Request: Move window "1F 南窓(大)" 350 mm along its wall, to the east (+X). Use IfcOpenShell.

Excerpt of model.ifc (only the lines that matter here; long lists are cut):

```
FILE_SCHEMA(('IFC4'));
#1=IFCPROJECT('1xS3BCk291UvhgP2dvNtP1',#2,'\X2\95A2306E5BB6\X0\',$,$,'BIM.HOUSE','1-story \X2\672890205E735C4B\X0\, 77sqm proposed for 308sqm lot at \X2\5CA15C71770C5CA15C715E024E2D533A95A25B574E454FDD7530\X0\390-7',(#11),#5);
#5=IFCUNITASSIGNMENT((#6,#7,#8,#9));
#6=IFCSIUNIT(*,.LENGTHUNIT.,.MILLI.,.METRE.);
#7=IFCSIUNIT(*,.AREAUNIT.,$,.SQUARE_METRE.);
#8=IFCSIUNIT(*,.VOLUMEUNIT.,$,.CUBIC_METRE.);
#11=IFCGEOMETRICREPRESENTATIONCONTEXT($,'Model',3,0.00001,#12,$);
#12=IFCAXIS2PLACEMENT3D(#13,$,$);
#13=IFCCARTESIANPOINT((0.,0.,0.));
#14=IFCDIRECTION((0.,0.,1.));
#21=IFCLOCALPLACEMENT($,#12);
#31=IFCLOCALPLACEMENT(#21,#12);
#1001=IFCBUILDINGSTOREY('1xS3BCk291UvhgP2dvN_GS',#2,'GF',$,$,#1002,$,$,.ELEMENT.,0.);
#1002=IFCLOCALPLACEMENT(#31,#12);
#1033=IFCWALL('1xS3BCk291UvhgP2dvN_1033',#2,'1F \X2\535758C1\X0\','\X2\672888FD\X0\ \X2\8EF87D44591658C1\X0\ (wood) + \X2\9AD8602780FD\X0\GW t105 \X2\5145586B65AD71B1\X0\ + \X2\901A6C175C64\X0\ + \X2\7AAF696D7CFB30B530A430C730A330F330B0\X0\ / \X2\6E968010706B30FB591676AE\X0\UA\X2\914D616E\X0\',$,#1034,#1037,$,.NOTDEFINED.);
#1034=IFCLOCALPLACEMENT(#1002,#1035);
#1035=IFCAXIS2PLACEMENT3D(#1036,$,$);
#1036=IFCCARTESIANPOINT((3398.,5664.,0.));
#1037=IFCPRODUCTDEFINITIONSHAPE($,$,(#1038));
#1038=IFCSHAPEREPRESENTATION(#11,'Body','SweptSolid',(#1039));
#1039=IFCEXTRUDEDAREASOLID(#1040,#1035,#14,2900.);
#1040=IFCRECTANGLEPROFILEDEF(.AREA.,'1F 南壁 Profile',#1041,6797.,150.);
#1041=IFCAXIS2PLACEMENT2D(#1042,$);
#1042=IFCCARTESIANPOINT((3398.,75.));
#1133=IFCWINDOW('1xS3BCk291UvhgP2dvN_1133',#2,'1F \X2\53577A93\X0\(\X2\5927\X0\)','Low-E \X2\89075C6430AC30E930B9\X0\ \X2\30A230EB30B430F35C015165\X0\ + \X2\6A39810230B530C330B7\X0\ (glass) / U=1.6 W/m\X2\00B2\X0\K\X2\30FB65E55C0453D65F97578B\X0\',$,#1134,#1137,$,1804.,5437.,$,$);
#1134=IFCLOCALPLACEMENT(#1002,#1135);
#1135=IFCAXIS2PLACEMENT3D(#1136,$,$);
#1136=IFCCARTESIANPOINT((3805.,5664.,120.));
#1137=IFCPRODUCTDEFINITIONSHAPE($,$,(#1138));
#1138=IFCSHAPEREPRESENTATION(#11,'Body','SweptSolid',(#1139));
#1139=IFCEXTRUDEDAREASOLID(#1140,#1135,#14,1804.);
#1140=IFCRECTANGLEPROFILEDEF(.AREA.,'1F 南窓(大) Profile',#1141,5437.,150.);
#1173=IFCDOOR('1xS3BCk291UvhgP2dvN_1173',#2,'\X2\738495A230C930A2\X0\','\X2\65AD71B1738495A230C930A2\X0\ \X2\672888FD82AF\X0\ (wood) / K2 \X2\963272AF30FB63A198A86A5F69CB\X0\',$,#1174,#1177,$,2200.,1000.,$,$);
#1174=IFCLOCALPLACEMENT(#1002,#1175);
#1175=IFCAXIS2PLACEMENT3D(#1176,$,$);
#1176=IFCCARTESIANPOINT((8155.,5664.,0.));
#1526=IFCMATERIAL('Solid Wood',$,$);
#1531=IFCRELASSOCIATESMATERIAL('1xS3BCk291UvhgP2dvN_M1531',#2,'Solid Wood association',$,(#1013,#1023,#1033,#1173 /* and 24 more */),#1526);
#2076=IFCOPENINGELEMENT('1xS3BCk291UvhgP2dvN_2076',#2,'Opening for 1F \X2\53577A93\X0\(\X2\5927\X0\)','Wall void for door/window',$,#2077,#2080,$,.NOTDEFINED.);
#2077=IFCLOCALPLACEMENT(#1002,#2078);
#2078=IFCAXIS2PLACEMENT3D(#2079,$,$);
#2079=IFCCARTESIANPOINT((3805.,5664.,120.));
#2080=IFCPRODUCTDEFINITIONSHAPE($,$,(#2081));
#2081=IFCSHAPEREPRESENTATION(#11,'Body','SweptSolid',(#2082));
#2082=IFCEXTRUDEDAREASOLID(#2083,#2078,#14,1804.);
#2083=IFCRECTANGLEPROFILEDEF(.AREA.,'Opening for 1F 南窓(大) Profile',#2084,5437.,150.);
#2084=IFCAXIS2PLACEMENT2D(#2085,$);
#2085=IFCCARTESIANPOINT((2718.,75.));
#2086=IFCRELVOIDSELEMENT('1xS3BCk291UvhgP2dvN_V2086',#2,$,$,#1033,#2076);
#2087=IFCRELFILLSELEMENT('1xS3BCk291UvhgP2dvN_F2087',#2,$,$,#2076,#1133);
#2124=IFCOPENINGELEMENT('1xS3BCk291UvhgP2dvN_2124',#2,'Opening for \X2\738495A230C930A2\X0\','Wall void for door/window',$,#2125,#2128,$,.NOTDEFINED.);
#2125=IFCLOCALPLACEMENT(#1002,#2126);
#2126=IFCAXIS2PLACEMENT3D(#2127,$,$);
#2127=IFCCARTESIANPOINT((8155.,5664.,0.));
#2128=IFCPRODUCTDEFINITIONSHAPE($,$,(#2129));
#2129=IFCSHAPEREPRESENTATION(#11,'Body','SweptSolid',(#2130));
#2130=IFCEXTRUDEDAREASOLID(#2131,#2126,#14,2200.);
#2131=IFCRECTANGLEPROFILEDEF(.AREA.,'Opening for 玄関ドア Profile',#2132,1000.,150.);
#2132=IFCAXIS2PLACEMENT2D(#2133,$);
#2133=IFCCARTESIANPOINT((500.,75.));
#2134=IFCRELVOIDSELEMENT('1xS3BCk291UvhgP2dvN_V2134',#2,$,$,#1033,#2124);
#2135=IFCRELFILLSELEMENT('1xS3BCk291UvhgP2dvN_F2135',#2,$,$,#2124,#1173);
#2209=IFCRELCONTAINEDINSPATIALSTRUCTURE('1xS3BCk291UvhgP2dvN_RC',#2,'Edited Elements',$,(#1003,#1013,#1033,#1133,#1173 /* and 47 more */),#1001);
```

```python
import ifcopenshell
import ifcopenshell.api.geometry
import ifcopenshell.util.placement

model = ifcopenshell.open("model.ifc")

window = model.by_guid("1xS3BCk291UvhgP2dvN_1133")
opening = window.FillsVoids[0].RelatingOpeningElement
wall = opening.VoidsElements[0].RelatingBuildingElement

wall_matrix = ifcopenshell.util.placement.get_local_placement(wall.ObjectPlacement)
shift = wall_matrix[:3, 0] * 350.0
before = ifcopenshell.util.placement.get_local_placement(window.ObjectPlacement)[:3, 3].copy()

# The window is not placed relative to its opening, so move both.
for product in (opening, window):
    matrix = ifcopenshell.util.placement.get_local_placement(product.ObjectPlacement)
    matrix[:3, 3] += shift
    ifcopenshell.api.geometry.edit_object_placement(model, product=product, matrix=matrix, is_si=False)

after = ifcopenshell.util.placement.get_local_placement(window.ObjectPlacement)[:3, 3]
print("window moved by", (after - before).round(3) + 0.0)

model.write("model_updated.ifc")
```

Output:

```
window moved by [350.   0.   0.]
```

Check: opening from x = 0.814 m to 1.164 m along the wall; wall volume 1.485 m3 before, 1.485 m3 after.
